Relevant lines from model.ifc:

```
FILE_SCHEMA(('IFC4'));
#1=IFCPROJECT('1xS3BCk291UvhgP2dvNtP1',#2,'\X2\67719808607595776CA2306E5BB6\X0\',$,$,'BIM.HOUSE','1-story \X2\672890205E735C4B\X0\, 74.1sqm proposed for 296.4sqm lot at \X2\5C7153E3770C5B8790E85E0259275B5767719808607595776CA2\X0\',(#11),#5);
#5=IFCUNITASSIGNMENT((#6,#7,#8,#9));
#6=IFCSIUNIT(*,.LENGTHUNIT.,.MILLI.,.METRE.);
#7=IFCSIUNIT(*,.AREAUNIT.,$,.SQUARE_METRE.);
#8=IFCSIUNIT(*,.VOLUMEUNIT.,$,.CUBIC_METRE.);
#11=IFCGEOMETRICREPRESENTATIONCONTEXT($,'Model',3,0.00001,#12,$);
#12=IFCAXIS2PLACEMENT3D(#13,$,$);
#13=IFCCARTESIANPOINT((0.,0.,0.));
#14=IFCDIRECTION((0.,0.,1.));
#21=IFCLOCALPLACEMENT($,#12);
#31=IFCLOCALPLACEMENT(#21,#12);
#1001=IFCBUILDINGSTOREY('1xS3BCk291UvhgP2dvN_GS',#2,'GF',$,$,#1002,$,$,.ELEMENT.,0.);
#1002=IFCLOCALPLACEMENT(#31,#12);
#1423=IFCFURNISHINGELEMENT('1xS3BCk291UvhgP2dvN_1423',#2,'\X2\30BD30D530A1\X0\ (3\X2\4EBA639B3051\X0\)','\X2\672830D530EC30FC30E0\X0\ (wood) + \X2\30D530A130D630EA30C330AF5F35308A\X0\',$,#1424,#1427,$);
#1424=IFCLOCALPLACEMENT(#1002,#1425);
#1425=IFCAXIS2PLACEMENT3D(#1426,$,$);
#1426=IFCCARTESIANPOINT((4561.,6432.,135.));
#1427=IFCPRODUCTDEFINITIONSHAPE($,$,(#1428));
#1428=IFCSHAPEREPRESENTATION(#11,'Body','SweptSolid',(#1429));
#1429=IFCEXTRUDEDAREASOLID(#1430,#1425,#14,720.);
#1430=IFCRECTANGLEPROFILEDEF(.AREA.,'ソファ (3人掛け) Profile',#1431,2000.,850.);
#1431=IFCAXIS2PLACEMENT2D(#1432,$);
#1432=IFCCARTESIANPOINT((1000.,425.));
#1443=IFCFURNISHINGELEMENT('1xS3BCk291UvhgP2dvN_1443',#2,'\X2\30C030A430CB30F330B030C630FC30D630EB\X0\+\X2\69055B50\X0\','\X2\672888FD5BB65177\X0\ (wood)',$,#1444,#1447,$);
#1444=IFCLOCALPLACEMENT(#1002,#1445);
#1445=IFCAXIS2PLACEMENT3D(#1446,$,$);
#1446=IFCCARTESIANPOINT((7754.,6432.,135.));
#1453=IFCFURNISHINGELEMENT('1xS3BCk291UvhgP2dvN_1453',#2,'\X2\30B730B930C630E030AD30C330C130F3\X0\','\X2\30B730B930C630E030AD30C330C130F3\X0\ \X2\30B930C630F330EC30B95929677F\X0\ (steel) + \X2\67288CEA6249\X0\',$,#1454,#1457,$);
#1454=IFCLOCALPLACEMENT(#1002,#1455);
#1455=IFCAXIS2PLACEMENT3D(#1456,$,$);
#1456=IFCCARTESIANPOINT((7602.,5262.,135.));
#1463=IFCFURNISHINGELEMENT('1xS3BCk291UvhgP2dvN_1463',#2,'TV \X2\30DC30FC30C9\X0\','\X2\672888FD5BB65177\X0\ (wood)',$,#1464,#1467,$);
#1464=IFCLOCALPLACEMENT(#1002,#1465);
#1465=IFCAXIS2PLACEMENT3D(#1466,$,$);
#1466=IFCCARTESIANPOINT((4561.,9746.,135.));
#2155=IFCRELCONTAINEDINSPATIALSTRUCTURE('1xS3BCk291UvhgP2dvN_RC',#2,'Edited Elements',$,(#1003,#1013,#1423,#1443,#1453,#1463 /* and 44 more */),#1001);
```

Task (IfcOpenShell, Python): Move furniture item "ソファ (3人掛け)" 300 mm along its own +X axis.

```python
import ifcopenshell
import ifcopenshell.api.geometry
import ifcopenshell.util.placement

model = ifcopenshell.open("model.ifc")

item = model.by_guid("1xS3BCk291UvhgP2dvN_1423")
matrix = ifcopenshell.util.placement.get_local_placement(item.ObjectPlacement)
matrix[:3, 3] += matrix[:3, 0] * 300.0
ifcopenshell.api.geometry.edit_object_placement(model, product=item, matrix=matrix, is_si=False)

print(ifcopenshell.util.placement.get_local_placement(item.ObjectPlacement).round(3) + 0.0)

model.write("model_edited.ifc")
```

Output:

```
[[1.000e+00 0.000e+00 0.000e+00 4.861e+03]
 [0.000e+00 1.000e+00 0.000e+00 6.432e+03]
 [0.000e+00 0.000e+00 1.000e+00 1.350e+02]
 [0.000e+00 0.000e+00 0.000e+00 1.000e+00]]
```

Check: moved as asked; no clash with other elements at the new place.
